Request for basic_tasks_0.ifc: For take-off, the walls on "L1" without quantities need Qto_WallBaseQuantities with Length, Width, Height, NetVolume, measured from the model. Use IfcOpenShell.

First a look at what the model holds.

```python
import ifcopenshell
import ifcopenshell.util.element
import ifcopenshell.util.unit

model = ifcopenshell.open("basic_tasks_0.ifc")
print(model.schema)
for unit_type in ("LENGTHUNIT", "AREAUNIT", "VOLUMEUNIT"):
    print(unit_type, ifcopenshell.util.unit.calculate_unit_scale(model, unit_type))
storey = next(s for s in model.by_type("IfcBuildingStorey") if s.Name == "L1")
walls = [e for e in ifcopenshell.util.element.get_decomposition(storey) if e.is_a("IfcWall")]
for e in sorted(walls, key=lambda e: e.id()):
    print(e.id(), e.is_a(), e.Name, list(ifcopenshell.util.element.get_psets(e, qtos_only=True)), sep=" | ")
```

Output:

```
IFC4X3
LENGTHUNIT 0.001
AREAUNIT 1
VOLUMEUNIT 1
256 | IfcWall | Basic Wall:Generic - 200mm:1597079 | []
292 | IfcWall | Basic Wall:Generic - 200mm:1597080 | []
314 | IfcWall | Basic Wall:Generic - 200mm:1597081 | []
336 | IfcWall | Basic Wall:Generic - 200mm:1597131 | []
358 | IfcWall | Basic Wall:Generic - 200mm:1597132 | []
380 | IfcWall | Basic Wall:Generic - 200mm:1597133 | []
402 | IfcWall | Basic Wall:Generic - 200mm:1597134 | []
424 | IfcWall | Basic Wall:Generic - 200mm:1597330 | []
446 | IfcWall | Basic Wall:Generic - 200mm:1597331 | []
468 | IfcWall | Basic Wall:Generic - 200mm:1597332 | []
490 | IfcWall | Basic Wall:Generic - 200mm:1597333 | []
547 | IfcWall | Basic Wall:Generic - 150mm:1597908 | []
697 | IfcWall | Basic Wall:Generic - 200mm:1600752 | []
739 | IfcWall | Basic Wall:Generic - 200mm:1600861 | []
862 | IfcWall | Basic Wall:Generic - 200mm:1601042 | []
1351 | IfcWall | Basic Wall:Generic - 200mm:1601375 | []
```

```python
import ifcopenshell
import ifcopenshell.api.pset
import ifcopenshell.geom
import ifcopenshell.util.element
import ifcopenshell.util.shape
import ifcopenshell.util.unit

model = ifcopenshell.open("basic_tasks_0.ifc")
unit_scale = ifcopenshell.util.unit.calculate_unit_scale(model)
volume_scale = ifcopenshell.util.unit.calculate_unit_scale(model, "VOLUMEUNIT")
settings = ifcopenshell.geom.settings()

storey = next(s for s in model.by_type("IfcBuildingStorey") if s.Name == "L1")
walls = [e for e in ifcopenshell.util.element.get_decomposition(storey) if e.is_a("IfcWall")]

for e in sorted(walls, key=lambda e: e.id()):
    if ifcopenshell.util.element.get_psets(e, qtos_only=True, should_inherit=False):
        continue
    # Geometry comes back in metres, in the element's own axes.
    shape = ifcopenshell.geom.create_shape(settings, e)
    values = {
        "Length": ifcopenshell.util.shape.get_x(shape.geometry) / unit_scale,
        "Width": ifcopenshell.util.shape.get_y(shape.geometry) / unit_scale,
        "Height": ifcopenshell.util.shape.get_z(shape.geometry) / unit_scale,
        "NetVolume": ifcopenshell.util.shape.get_volume(shape.geometry) / volume_scale,
    }
    qto = ifcopenshell.api.pset.add_qto(model, product=e, name="Qto_WallBaseQuantities")
    ifcopenshell.api.pset.edit_qto(model, qto=qto, properties=values)
    print(e.id(), {k: round(v, 3) for k, v in values.items()})

model.write("basic_tasks_0_edited.ifc")
```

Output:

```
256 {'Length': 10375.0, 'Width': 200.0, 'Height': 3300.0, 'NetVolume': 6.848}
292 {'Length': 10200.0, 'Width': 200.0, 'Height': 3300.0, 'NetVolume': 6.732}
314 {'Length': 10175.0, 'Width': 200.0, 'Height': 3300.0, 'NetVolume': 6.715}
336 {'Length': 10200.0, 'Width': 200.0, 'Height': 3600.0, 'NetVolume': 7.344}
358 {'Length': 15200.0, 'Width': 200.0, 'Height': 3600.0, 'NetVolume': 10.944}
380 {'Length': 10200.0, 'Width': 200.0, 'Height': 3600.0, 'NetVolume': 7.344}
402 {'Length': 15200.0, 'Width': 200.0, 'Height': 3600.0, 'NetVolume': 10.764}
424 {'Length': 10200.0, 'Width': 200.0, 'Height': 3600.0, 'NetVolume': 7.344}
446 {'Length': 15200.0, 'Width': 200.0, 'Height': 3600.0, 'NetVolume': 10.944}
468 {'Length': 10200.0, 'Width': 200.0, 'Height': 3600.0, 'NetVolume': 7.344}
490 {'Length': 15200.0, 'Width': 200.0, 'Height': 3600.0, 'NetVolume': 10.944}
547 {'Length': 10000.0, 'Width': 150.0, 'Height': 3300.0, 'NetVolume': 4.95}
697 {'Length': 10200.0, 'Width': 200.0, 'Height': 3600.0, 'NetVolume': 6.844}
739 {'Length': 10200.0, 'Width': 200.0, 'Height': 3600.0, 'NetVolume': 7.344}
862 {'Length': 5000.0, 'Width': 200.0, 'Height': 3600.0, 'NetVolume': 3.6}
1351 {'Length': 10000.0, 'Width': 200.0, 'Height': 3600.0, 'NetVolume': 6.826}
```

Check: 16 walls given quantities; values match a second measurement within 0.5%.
